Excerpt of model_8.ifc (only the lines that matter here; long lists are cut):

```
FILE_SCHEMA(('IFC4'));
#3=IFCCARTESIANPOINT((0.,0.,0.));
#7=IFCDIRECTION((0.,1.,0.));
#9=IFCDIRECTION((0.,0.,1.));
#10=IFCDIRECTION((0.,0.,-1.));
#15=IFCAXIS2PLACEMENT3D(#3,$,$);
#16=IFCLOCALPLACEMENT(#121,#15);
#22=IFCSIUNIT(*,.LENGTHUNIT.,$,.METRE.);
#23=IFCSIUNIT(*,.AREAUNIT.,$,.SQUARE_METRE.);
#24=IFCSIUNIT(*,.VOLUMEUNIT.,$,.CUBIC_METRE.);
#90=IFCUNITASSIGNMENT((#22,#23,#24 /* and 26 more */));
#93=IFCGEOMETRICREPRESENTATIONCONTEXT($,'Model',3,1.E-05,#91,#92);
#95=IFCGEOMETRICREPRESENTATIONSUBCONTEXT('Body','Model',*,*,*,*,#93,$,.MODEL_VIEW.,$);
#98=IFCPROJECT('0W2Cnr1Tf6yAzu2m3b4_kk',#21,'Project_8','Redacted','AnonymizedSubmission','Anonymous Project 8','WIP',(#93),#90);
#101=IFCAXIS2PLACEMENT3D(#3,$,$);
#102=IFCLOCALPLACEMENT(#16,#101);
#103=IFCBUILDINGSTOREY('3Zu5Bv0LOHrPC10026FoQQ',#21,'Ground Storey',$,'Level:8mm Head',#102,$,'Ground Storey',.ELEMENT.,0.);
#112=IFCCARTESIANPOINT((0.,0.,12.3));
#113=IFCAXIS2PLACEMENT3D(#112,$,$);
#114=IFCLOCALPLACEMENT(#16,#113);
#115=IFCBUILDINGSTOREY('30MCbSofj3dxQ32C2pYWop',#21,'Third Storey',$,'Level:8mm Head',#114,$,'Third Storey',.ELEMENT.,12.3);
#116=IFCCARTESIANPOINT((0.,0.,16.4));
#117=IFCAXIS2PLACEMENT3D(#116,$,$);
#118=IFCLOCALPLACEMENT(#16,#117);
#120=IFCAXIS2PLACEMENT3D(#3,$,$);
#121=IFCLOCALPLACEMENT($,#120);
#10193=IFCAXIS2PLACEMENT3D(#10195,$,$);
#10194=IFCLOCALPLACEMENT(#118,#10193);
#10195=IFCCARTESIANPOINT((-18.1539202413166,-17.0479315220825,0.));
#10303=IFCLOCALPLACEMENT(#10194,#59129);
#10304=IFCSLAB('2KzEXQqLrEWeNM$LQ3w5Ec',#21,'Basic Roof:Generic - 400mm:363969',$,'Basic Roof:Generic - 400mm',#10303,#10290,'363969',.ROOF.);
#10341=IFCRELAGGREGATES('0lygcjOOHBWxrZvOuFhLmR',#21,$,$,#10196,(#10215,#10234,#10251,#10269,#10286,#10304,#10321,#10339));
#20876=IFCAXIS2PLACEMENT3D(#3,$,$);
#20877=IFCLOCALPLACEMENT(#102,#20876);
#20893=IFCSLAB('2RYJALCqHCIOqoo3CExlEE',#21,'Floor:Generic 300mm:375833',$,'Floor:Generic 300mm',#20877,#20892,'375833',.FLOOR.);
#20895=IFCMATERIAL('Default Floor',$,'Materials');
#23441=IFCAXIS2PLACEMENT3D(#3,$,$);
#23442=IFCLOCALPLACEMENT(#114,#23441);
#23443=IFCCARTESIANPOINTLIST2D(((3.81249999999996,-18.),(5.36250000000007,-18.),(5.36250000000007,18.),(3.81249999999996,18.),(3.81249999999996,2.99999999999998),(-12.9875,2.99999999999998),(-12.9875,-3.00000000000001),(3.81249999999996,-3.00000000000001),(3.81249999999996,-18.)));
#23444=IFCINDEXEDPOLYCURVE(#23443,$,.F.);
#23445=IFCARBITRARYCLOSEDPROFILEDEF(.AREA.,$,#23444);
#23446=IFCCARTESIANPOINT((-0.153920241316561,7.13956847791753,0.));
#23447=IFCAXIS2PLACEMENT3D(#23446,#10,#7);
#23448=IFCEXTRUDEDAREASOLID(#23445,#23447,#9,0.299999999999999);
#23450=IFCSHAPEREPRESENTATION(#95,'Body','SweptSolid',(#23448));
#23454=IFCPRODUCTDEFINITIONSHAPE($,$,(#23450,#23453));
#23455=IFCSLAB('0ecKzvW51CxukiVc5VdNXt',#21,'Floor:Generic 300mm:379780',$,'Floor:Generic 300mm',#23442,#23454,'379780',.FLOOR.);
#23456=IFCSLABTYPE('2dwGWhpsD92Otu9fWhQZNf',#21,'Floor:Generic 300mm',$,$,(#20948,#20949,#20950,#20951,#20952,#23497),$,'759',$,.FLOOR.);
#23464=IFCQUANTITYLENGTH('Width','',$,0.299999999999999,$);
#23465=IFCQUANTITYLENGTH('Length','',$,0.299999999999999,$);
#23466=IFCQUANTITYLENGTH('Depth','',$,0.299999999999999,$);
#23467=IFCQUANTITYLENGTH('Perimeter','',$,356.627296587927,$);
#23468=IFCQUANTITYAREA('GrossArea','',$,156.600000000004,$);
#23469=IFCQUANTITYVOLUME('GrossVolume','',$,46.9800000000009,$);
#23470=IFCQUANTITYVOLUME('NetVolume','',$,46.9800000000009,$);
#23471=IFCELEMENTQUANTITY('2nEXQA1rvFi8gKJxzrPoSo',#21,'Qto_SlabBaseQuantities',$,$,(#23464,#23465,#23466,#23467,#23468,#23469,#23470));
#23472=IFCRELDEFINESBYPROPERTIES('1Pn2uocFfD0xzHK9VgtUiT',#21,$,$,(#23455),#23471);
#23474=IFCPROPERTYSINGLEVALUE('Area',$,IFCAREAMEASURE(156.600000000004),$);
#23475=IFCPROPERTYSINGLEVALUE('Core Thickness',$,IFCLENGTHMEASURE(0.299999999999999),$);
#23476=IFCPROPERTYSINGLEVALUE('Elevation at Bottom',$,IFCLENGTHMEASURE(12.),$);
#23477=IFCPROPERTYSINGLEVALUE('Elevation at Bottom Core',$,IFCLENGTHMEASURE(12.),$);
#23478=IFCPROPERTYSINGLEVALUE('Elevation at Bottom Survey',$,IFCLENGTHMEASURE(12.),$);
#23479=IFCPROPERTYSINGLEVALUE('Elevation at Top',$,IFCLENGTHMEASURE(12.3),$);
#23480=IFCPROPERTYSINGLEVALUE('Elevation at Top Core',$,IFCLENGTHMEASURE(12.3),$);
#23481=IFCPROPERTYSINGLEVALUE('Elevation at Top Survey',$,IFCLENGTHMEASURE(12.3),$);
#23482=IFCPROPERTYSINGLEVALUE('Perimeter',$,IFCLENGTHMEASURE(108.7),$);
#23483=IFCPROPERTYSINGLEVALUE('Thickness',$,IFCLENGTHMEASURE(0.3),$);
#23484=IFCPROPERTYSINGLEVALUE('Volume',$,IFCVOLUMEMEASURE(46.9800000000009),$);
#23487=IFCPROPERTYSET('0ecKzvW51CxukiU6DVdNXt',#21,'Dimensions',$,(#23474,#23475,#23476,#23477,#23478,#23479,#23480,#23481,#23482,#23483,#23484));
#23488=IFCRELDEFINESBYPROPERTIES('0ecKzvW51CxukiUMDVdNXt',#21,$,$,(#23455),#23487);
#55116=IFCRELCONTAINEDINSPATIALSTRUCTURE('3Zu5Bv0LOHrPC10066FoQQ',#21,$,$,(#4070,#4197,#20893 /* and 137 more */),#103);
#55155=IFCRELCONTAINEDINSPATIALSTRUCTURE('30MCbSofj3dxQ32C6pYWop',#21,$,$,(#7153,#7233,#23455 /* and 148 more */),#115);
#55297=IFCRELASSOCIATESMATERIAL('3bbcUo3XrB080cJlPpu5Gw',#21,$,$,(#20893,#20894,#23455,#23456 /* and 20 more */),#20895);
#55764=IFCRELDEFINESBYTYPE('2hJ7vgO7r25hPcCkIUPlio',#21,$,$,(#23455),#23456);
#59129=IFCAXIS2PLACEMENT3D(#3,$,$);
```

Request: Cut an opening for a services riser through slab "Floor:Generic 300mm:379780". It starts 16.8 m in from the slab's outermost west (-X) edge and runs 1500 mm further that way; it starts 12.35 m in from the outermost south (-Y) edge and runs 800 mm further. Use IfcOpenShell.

```python
import numpy as np
import ifcopenshell
import ifcopenshell.api.feature
import ifcopenshell.api.geometry
import ifcopenshell.api.pset
import ifcopenshell.api.root
import ifcopenshell.geom
import ifcopenshell.util.element
import ifcopenshell.util.placement
import ifcopenshell.util.representation
import ifcopenshell.util.shape
import ifcopenshell.util.unit

model = ifcopenshell.open("model_8.ifc")
unit_scale = ifcopenshell.util.unit.calculate_unit_scale(model)
area_scale = ifcopenshell.util.unit.calculate_unit_scale(model, "AREAUNIT")
volume_scale = ifcopenshell.util.unit.calculate_unit_scale(model, "VOLUMEUNIT")
settings = ifcopenshell.geom.settings()


def volume(element):
    """Net volume in cubic metres, openings subtracted."""
    shape = ifcopenshell.geom.create_shape(settings, element)
    return ifcopenshell.util.shape.get_volume(shape.geometry)


slab = model.by_id(23455)
before = volume(slab)

# Extent in the slab's own axes, in metres. The edges named are its -X and -Y sides.
slab_shape = ifcopenshell.geom.create_shape(settings, slab)
vertices = ifcopenshell.util.shape.get_vertices(slab_shape.geometry)
x_min, y_min, bottom = vertices.min(axis=0)
top = vertices[:, 2].max()

opening = ifcopenshell.api.root.create_entity(model, ifc_class="IfcOpeningElement", name="Services riser opening", predefined_type="OPENING")
context = ifcopenshell.util.representation.get_context(model, "Model", "Body", "MODEL_VIEW")
width, depth = 1.5, 0.8
outline = [(0.0, 0.0), (width, 0.0), (width, depth), (0.0, depth), (0.0, 0.0)]
# Overshoot both faces by 50 mm so the cut is clean.
shape = ifcopenshell.api.geometry.add_slab_representation(
    model, context=context, depth=top - bottom + 0.1, polyline=outline
)
ifcopenshell.api.geometry.assign_representation(model, product=opening, representation=shape)

matrix = ifcopenshell.util.placement.get_local_placement(slab.ObjectPlacement)
matrix[:, 3] = matrix @ np.append(np.array([x_min + 16.8, y_min + 12.35, bottom - 0.05]) / unit_scale, 1.0)
ifcopenshell.api.geometry.edit_object_placement(model, product=opening, matrix=matrix, is_si=False)
ifcopenshell.api.feature.add_feature(model, feature=opening, element=slab)

after = volume(slab)

# Update the slab's stored quantities.
qto = model.by_id(ifcopenshell.util.element.get_pset(slab, "Qto_SlabBaseQuantities", should_inherit=False)["id"])
ifcopenshell.api.pset.edit_qto(model, qto=qto, properties={"NetVolume": after / volume_scale})
pset = model.by_id(ifcopenshell.util.element.get_pset(slab, "Dimensions", should_inherit=False)["id"])
ifcopenshell.api.pset.edit_pset(model, pset=pset, properties={
    "Area": model.create_entity("IfcAreaMeasure", after / (top - bottom) / area_scale),
    "Volume": model.create_entity("IfcVolumeMeasure", after / volume_scale),
})

print(f"slab volume {before:.3f} -> {after:.3f} m3")

model.write("model_8_v2.ifc")
```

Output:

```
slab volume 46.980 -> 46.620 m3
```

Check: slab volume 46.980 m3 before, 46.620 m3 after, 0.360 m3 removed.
